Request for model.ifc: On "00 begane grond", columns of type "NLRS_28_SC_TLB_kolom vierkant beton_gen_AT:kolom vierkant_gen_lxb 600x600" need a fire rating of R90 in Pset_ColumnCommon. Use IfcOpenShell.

First a look at what the model holds.

```python
import ifcopenshell
import ifcopenshell.util.element

model = ifcopenshell.open("model.ifc")
print(model.schema)
storey = next(s for s in model.by_type("IfcBuildingStorey") if s.Name == "00 begane grond")
columns = [e for e in ifcopenshell.util.element.get_decomposition(storey) if e.is_a("IfcColumn")]
seen = {}
for e in columns:
    element_type = ifcopenshell.util.element.get_type(e)
    key = (element_type.Name if element_type != e and element_type else None, ifcopenshell.util.element.get_pset(e, "Pset_ColumnCommon", "FireRating"))
    seen[key] = seen.get(key, 0) + 1
for (name, value), count in sorted(seen.items(), key=str):
    print(count, "x", name, "|", value)
```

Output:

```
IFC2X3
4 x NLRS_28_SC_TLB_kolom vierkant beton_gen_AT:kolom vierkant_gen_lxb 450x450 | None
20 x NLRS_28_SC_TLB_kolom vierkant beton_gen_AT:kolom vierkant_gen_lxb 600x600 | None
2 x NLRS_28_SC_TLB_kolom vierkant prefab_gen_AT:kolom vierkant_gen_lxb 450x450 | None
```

```python
import ifcopenshell
import ifcopenshell.api.pset
import ifcopenshell.util.element

model = ifcopenshell.open("model.ifc")

storey = next(s for s in model.by_type("IfcBuildingStorey") if s.Name == "00 begane grond")
columns = [e for e in ifcopenshell.util.element.get_decomposition(storey) if e.is_a("IfcColumn")]

count = 0
for e in columns:
    element_type = ifcopenshell.util.element.get_type(e)
    if element_type in (None, e) or element_type.Name != "NLRS_28_SC_TLB_kolom vierkant beton_gen_AT:kolom vierkant_gen_lxb 600x600":
        continue
    found = ifcopenshell.util.element.get_pset(e, "Pset_ColumnCommon", should_inherit=False)
    if found:
        pset = model.by_id(found["id"])
        if len(ifcopenshell.util.element.get_elements_by_pset(pset)) > 1:
            pset = ifcopenshell.api.pset.unshare_pset(model, products=[e], pset=pset)[0]
    else:
        pset = ifcopenshell.api.pset.add_pset(model, product=e, name="Pset_ColumnCommon")
    ifcopenshell.api.pset.edit_pset(model, pset=pset, properties={"FireRating": "R90"})
    count += 1

print(count, "columns updated")

model.write("model_rev.ifc")
```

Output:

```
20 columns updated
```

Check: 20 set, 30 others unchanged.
